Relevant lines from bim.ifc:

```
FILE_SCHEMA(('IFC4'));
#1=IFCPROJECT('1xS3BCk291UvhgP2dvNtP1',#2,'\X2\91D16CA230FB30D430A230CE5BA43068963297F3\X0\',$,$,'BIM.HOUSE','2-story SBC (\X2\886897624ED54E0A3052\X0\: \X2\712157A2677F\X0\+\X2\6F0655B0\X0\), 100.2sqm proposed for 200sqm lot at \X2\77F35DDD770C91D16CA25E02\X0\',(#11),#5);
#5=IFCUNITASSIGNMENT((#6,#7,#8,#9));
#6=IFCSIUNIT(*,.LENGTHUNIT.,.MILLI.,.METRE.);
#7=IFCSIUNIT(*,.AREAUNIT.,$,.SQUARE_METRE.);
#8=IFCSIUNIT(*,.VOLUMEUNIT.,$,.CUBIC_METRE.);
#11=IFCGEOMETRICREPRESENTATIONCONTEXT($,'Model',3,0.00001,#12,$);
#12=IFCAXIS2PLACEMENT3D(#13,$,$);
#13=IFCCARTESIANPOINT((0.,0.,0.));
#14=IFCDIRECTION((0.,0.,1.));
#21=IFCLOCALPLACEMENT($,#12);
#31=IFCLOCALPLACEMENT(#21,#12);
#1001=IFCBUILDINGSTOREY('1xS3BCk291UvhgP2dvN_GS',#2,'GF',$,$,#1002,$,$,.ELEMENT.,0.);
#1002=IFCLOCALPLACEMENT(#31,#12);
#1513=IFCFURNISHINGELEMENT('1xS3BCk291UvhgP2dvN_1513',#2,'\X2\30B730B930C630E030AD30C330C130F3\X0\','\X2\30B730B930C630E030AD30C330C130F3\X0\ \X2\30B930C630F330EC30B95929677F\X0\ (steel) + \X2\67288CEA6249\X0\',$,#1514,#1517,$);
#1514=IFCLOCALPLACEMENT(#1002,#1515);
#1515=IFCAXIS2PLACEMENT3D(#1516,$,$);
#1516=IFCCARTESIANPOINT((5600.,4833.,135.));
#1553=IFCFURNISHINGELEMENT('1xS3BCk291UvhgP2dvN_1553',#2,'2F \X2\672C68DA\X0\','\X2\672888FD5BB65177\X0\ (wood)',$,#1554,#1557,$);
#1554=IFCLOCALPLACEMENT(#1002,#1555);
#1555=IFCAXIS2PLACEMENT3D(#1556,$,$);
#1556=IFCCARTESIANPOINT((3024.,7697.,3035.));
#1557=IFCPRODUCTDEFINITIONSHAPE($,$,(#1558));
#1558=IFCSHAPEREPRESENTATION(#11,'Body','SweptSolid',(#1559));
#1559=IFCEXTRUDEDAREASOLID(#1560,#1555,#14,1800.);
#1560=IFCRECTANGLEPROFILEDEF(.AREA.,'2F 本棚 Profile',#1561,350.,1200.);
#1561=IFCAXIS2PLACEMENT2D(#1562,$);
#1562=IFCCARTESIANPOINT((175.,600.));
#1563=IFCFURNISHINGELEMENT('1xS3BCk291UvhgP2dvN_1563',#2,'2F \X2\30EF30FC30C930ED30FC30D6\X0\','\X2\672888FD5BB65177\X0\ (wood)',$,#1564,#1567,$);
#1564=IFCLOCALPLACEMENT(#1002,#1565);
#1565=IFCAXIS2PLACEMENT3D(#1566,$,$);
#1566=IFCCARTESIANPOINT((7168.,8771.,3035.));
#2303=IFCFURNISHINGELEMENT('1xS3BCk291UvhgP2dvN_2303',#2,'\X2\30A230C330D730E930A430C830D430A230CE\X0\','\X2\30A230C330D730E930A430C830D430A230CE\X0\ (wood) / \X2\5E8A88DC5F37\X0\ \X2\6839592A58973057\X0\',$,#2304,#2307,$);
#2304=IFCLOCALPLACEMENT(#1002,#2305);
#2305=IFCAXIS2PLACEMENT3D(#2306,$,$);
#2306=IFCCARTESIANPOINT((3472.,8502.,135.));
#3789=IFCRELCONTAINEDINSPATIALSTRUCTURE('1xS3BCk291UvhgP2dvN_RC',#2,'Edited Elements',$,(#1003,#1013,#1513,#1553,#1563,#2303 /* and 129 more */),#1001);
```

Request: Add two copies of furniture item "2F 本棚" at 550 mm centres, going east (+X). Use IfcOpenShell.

```python
import numpy as np
import ifcopenshell
import ifcopenshell.api.geometry
import ifcopenshell.api.root
import ifcopenshell.util.element
import ifcopenshell.util.placement

model = ifcopenshell.open("bim.ifc")


def reuse_history(source, copy):
    """copy_class also copies each property set's owner history, people and application; keep the originals."""
    for rel in copy.IsDefinedBy:
        if rel.is_a("IfcRelDefinesByProperties") and (history := rel.RelatingPropertyDefinition.OwnerHistory):
            rel.RelatingPropertyDefinition.OwnerHistory = source.OwnerHistory
            ifcopenshell.util.element.remove_deep2(model, history)


source = model.by_guid("1xS3BCk291UvhgP2dvN_1553")
base = ifcopenshell.util.placement.get_local_placement(source.ObjectPlacement)
step = np.array([1.0, 0.0, 0.0]) * 550.0

for i in range(1, 3):
    copy = ifcopenshell.api.root.copy_class(model, product=source)
    copy.Representation = ifcopenshell.util.element.copy_deep(
        model, source.Representation, exclude=["IfcGeometricRepresentationContext", "IfcRepresentationMap"]
    )
    reuse_history(source, copy)
    matrix = base.copy()
    matrix[:3, 3] += i * step
    print("added at", matrix[:3, 3].round(3) + 0.0)
    ifcopenshell.api.geometry.edit_object_placement(model, product=copy, matrix=matrix, is_si=False)

model.write("bim_v2.ifc")
```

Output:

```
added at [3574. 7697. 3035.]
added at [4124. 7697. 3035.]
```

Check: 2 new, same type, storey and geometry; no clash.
